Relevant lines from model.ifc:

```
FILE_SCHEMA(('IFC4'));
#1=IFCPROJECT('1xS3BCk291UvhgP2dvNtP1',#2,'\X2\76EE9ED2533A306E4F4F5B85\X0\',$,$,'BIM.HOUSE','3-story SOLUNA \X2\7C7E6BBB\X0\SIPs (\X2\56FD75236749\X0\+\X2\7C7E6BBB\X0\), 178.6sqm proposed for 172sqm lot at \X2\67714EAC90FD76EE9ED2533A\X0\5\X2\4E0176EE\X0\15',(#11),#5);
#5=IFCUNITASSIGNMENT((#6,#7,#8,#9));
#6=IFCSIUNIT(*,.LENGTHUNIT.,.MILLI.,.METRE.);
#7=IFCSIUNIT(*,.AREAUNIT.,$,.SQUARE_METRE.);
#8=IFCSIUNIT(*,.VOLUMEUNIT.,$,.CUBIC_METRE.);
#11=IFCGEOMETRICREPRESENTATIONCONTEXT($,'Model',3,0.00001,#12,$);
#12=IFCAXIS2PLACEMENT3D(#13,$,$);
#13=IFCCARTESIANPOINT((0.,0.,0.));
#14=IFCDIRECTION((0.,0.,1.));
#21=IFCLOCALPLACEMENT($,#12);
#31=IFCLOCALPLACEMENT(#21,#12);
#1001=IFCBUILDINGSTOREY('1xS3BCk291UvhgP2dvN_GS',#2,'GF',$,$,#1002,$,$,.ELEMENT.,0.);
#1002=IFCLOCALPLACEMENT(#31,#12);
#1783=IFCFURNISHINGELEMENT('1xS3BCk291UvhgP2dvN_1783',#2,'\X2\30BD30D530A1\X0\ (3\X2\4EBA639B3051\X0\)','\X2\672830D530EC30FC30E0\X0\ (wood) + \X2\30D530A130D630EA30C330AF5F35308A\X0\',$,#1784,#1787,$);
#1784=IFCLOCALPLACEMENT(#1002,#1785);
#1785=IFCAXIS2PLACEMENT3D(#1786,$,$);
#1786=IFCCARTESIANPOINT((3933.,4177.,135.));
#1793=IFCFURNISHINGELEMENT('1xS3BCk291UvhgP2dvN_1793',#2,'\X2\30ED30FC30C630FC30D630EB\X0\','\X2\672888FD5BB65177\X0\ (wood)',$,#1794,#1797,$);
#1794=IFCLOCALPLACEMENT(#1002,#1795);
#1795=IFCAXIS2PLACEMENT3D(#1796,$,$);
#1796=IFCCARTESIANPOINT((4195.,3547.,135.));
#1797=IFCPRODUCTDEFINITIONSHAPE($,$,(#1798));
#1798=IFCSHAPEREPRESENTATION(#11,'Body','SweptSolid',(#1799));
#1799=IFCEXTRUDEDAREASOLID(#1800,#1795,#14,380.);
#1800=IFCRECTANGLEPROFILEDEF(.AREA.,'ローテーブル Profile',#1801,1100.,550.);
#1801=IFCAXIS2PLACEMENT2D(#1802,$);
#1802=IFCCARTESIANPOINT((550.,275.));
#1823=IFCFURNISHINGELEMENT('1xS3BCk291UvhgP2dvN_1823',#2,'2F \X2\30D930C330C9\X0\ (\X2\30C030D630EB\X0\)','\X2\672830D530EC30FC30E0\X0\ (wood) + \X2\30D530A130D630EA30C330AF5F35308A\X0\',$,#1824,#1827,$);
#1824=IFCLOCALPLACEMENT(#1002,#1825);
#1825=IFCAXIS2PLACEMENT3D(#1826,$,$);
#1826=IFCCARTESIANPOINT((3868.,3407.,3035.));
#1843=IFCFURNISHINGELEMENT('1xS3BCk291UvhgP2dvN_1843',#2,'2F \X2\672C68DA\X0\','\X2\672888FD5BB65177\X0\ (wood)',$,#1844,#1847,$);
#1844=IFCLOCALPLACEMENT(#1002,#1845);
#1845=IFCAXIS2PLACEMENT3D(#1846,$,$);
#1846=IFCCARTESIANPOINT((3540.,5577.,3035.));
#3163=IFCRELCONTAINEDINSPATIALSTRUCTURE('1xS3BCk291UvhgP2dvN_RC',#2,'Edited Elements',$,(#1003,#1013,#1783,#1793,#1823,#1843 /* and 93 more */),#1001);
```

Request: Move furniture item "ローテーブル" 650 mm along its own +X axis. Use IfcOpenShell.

```python
import ifcopenshell
import ifcopenshell.api.geometry
import ifcopenshell.util.placement

model = ifcopenshell.open("model.ifc")

item = model.by_id(1793)
matrix = ifcopenshell.util.placement.get_local_placement(item.ObjectPlacement)
matrix[:3, 3] += matrix[:3, 0] * 650.0
ifcopenshell.api.geometry.edit_object_placement(model, product=item, matrix=matrix, is_si=False)

print(ifcopenshell.util.placement.get_local_placement(item.ObjectPlacement).round(3) + 0.0)

model.write("model_edited.ifc")
```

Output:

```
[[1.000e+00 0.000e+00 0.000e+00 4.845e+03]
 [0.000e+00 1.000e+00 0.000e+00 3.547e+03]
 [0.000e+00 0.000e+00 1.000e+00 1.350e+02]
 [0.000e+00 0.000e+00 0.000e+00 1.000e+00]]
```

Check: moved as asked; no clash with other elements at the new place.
